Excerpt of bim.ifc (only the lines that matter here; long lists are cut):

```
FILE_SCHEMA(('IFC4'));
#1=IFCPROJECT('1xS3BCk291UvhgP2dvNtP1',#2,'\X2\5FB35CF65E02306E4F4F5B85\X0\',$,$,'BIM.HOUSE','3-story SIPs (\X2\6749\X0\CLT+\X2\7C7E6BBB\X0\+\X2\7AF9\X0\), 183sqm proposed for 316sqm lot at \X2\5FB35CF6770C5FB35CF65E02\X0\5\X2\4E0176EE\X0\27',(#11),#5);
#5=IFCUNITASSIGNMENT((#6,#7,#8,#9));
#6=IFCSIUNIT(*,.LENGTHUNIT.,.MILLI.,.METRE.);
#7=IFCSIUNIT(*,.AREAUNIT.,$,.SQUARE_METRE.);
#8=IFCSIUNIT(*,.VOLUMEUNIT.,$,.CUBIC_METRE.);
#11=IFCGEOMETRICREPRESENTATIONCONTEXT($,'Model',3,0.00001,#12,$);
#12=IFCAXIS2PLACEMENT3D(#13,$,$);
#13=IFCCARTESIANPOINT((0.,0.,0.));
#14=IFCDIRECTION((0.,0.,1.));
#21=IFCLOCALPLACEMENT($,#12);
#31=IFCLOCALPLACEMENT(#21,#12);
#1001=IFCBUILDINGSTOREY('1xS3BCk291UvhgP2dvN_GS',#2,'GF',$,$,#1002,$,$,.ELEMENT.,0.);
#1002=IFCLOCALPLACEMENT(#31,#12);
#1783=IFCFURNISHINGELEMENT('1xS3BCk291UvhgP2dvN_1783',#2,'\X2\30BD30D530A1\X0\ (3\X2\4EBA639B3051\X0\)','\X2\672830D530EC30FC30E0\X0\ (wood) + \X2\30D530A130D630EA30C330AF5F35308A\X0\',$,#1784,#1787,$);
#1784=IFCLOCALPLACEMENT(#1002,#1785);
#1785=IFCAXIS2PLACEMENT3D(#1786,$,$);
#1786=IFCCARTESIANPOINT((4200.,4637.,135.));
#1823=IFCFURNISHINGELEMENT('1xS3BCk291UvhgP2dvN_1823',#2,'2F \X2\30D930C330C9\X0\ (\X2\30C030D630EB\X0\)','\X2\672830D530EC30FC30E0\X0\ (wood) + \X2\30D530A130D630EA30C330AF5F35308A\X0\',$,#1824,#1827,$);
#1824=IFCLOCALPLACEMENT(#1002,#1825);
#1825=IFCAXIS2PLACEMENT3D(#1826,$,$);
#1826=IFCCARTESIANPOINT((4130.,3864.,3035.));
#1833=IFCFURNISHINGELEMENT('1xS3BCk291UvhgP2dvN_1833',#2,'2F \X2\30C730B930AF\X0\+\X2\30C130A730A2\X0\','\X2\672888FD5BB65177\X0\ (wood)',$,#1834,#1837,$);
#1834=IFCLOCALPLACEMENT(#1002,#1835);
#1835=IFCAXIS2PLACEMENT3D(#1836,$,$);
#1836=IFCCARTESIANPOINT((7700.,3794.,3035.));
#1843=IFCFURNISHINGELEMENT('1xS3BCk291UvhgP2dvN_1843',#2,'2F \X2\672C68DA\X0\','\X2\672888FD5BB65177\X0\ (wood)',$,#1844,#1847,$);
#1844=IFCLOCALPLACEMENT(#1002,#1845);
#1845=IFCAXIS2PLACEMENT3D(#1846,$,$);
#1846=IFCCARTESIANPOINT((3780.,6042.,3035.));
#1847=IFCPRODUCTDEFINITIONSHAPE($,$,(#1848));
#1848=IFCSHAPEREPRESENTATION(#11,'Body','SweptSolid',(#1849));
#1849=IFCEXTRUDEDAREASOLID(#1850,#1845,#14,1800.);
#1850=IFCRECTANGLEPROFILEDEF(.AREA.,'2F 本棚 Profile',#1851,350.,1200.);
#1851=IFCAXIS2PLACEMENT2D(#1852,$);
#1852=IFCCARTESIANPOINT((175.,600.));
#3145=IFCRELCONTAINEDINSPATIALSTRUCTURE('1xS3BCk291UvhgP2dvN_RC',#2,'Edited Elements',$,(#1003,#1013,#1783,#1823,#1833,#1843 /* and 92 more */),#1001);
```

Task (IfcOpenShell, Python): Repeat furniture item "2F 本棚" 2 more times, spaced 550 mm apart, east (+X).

```python
import numpy as np
import ifcopenshell
import ifcopenshell.api.geometry
import ifcopenshell.api.root
import ifcopenshell.util.element
import ifcopenshell.util.placement
import ifcopenshell.util.unit

model = ifcopenshell.open("bim.ifc")
unit_scale = ifcopenshell.util.unit.calculate_unit_scale(model)


def reuse_history(source, copy):
    """copy_class also copies each property set's owner history, people and application; keep the originals."""
    for rel in copy.IsDefinedBy:
        if rel.is_a("IfcRelDefinesByProperties") and (history := rel.RelatingPropertyDefinition.OwnerHistory):
            rel.RelatingPropertyDefinition.OwnerHistory = source.OwnerHistory
            ifcopenshell.util.element.remove_deep2(model, history)


source = model.by_guid("1xS3BCk291UvhgP2dvN_1843")
base = ifcopenshell.util.placement.get_local_placement(source.ObjectPlacement)
step = np.array([1.0, 0.0, 0.0]) * 0.55 / unit_scale

for i in range(1, 3):
    copy = ifcopenshell.api.root.copy_class(model, product=source)
    copy.Representation = ifcopenshell.util.element.copy_deep(
        model, source.Representation, exclude=["IfcGeometricRepresentationContext", "IfcRepresentationMap"]
    )
    reuse_history(source, copy)
    matrix = base.copy()
    matrix[:3, 3] += i * step
    print("added at", matrix[:3, 3].round(3) + 0.0)
    ifcopenshell.api.geometry.edit_object_placement(model, product=copy, matrix=matrix, is_si=False)

model.write("bim_updated.ifc")
```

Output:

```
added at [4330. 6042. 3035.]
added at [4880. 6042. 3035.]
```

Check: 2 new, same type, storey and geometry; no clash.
